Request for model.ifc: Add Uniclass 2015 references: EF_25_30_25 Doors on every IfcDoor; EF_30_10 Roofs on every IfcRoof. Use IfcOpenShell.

First a look at what the model holds.

```python
import ifcopenshell

model = ifcopenshell.open("model.ifc")
print(model.schema)
print("classifications:", [c.Name for c in model.by_type("IfcClassification")])
for ifc_class in ("IfcDoor", "IfcRoof", "IfcStair", "IfcWall", "IfcWindow"):
    print(ifc_class, len(model.by_type(ifc_class)))
```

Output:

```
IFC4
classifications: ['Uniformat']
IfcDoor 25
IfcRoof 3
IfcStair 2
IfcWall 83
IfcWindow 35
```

```python
import ifcopenshell
import ifcopenshell.api.classification

model = ifcopenshell.open("model.ifc")

system = ifcopenshell.api.classification.add_classification(model, classification="Uniclass 2015")

codes = {
    "IfcDoor": ("EF_25_30_25", "Doors"),
    "IfcRoof": ("EF_30_10", "Roofs"),
}
for ifc_class, (code, name) in codes.items():
    products = model.by_type(ifc_class)
    ifcopenshell.api.classification.add_reference(
        model, products=products, classification=system, identification=code, name=name
    )
    print(code, len(products))

model.write("model_updated.ifc")
```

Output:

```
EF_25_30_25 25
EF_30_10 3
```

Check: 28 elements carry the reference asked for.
